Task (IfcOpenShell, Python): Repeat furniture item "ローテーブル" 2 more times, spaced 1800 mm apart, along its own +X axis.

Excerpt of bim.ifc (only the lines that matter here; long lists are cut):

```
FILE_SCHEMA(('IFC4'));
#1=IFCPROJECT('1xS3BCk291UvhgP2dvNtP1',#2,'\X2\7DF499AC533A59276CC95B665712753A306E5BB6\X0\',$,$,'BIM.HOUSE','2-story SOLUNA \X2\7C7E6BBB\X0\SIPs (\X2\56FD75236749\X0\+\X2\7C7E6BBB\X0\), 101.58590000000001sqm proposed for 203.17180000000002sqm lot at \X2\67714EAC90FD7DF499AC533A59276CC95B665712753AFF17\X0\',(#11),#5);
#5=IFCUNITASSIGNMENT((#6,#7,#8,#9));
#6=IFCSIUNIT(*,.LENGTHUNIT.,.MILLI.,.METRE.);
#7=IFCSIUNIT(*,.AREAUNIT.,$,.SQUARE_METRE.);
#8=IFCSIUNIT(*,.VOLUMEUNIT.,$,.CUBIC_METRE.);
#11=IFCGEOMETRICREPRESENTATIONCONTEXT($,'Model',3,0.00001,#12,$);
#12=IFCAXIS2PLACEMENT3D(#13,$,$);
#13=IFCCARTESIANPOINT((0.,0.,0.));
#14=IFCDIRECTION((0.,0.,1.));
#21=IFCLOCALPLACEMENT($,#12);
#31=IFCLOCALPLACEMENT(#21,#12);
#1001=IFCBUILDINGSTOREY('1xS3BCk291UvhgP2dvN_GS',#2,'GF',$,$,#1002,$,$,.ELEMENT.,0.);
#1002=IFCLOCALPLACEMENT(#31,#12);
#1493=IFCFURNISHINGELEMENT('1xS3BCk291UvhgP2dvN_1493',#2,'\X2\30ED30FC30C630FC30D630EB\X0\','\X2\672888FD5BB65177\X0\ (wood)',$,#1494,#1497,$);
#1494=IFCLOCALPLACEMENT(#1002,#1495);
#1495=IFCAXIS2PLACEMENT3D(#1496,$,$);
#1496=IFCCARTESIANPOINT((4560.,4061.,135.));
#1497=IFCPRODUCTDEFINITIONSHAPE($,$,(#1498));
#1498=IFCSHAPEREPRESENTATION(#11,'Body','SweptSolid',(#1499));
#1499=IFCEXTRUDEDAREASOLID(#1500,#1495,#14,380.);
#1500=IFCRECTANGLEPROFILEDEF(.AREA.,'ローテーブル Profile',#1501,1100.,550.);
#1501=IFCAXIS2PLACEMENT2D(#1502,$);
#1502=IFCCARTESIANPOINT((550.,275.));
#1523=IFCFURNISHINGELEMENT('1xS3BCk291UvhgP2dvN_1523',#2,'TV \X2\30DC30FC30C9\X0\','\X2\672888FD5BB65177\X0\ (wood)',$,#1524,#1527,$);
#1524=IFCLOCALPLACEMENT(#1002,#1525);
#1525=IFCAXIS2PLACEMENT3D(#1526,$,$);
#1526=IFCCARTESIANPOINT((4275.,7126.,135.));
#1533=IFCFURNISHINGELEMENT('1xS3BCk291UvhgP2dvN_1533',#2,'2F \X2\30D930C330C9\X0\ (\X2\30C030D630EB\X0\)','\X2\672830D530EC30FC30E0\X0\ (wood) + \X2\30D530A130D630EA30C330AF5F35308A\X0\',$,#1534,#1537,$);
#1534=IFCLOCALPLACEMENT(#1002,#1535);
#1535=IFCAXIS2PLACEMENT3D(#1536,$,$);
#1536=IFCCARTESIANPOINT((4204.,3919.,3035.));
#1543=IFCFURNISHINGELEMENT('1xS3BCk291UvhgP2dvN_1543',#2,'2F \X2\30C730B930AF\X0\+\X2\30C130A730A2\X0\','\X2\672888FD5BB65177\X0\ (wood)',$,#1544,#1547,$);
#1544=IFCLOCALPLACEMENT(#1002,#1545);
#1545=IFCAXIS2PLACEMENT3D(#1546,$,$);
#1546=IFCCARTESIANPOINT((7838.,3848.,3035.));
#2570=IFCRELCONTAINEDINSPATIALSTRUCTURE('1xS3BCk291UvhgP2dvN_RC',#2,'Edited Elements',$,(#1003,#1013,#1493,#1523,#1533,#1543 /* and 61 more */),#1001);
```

```python
import ifcopenshell
import ifcopenshell.api.geometry
import ifcopenshell.api.root
import ifcopenshell.util.element
import ifcopenshell.util.placement

model = ifcopenshell.open("bim.ifc")


def reuse_history(source, copy):
    """copy_class also copies each property set's owner history, people and application; keep the originals."""
    for rel in copy.IsDefinedBy:
        if rel.is_a("IfcRelDefinesByProperties") and (history := rel.RelatingPropertyDefinition.OwnerHistory):
            rel.RelatingPropertyDefinition.OwnerHistory = source.OwnerHistory
            ifcopenshell.util.element.remove_deep2(model, history)


source = model.by_guid("1xS3BCk291UvhgP2dvN_1493")
base = ifcopenshell.util.placement.get_local_placement(source.ObjectPlacement)
step = base[:3, 0] * 1800.0

for i in range(1, 3):
    copy = ifcopenshell.api.root.copy_class(model, product=source)
    copy.Representation = ifcopenshell.util.element.copy_deep(
        model, source.Representation, exclude=["IfcGeometricRepresentationContext", "IfcRepresentationMap"]
    )
    reuse_history(source, copy)
    matrix = base.copy()
    matrix[:3, 3] += i * step
    print("added at", matrix[:3, 3].round(3) + 0.0)
    ifcopenshell.api.geometry.edit_object_placement(model, product=copy, matrix=matrix, is_si=False)

model.write("bim_edited.ifc")
```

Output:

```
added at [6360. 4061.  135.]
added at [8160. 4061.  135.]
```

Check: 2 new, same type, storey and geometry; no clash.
